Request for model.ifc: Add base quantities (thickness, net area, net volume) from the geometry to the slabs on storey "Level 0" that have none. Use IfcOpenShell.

First a look at what the model holds.

```python
import ifcopenshell
import ifcopenshell.util.element
import ifcopenshell.util.unit

model = ifcopenshell.open("model.ifc")
print(model.schema)
for unit_type in ("LENGTHUNIT", "AREAUNIT", "VOLUMEUNIT"):
    print(unit_type, ifcopenshell.util.unit.calculate_unit_scale(model, unit_type))
storey = next(s for s in model.by_type("IfcBuildingStorey") if s.Name == "Level 0")
slabs = [e for e in ifcopenshell.util.element.get_decomposition(storey) if e.is_a("IfcSlab")]
for e in sorted(slabs, key=lambda e: e.id()):
    print(e.id(), e.is_a(), e.Name, list(ifcopenshell.util.element.get_psets(e, qtos_only=True)), sep=" | ")
```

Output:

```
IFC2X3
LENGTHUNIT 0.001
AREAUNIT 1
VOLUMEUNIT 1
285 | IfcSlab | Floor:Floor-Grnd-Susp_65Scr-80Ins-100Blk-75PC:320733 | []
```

```python
import ifcopenshell
import ifcopenshell.api.pset
import ifcopenshell.geom
import ifcopenshell.util.element
import ifcopenshell.util.shape
import ifcopenshell.util.unit

model = ifcopenshell.open("model.ifc")
unit_scale = ifcopenshell.util.unit.calculate_unit_scale(model)
area_scale = ifcopenshell.util.unit.calculate_unit_scale(model, "AREAUNIT")
volume_scale = ifcopenshell.util.unit.calculate_unit_scale(model, "VOLUMEUNIT")
settings = ifcopenshell.geom.settings()

storey = next(s for s in model.by_type("IfcBuildingStorey") if s.Name == "Level 0")
slabs = [e for e in ifcopenshell.util.element.get_decomposition(storey) if e.is_a("IfcSlab")]

for e in sorted(slabs, key=lambda e: e.id()):
    if ifcopenshell.util.element.get_psets(e, qtos_only=True, should_inherit=False):
        continue
    # Geometry comes back in metres, in the element's own axes.
    shape = ifcopenshell.geom.create_shape(settings, e)
    values = {
        "Width": ifcopenshell.util.shape.get_z(shape.geometry) / unit_scale,
        "NetArea": ifcopenshell.util.shape.get_footprint_area(shape.geometry) / area_scale,
        "NetVolume": ifcopenshell.util.shape.get_volume(shape.geometry) / volume_scale,
    }
    qto = ifcopenshell.api.pset.add_qto(model, product=e, name="BaseQuantities")
    ifcopenshell.api.pset.edit_qto(model, qto=qto, properties=values)
    print(e.id(), {k: round(v, 3) for k, v in values.items()})

model.write("model_edited.ifc")
```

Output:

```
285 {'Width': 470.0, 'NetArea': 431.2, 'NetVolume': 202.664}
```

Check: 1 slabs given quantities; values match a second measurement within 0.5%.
